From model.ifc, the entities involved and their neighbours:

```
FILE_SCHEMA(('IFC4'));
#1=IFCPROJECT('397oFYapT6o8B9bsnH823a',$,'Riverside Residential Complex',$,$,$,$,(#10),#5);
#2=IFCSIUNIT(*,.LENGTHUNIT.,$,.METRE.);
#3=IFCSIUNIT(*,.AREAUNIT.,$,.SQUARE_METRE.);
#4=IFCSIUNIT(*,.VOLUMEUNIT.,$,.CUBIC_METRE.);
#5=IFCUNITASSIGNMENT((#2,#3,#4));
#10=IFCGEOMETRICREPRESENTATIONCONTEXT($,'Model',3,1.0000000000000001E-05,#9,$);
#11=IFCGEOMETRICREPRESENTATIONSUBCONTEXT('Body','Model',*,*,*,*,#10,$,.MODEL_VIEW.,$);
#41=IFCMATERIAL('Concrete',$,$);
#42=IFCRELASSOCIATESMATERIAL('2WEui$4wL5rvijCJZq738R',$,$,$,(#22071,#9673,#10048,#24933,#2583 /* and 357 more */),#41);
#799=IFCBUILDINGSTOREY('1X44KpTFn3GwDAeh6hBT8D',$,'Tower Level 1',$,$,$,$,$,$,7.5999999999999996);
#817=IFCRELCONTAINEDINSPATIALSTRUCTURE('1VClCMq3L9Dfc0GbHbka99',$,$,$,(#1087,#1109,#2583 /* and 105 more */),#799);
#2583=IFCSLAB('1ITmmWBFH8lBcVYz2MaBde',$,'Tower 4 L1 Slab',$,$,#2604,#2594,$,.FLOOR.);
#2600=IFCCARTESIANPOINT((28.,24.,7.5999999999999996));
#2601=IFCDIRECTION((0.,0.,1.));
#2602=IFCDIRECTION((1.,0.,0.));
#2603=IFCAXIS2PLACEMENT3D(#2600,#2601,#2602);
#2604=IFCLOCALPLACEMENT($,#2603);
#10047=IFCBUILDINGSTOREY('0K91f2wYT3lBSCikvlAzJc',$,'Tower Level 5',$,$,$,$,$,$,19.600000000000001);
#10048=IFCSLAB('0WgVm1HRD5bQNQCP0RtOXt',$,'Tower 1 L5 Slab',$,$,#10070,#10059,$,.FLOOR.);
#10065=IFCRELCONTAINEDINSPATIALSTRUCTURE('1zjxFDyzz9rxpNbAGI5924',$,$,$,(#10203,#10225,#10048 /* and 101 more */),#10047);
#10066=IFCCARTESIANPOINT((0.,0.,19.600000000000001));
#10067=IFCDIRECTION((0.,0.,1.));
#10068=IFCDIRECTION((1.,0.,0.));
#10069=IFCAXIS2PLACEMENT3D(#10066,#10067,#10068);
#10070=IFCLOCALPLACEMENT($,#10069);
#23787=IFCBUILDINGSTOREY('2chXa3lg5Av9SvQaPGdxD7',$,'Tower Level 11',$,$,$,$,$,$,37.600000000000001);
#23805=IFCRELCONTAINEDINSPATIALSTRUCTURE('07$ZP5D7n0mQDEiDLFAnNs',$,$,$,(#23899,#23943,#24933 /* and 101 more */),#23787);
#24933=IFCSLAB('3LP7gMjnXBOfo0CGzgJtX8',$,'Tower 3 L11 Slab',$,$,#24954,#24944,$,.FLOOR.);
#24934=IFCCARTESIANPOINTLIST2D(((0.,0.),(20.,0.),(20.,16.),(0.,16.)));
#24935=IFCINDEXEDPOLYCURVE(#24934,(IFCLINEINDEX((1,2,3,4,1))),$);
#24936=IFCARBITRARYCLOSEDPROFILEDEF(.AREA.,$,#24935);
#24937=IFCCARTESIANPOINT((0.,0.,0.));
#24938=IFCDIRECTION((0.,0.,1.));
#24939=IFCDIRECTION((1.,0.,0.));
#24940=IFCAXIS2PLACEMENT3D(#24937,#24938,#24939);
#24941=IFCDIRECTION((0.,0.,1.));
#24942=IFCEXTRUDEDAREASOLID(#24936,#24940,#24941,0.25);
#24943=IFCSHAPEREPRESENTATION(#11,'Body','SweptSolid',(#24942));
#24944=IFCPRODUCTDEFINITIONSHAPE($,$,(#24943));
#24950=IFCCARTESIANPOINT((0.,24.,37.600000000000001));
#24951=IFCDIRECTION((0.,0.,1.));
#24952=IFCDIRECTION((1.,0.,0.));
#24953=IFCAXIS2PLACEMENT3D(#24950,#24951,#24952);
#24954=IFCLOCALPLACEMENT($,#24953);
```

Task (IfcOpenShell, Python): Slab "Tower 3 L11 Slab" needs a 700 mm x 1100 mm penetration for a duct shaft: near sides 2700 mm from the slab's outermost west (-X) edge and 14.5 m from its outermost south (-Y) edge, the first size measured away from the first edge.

```python
import numpy as np
import ifcopenshell
import ifcopenshell.api.feature
import ifcopenshell.api.geometry
import ifcopenshell.api.root
import ifcopenshell.geom
import ifcopenshell.util.placement
import ifcopenshell.util.representation
import ifcopenshell.util.shape
import ifcopenshell.util.unit

model = ifcopenshell.open("model.ifc")
unit_scale = ifcopenshell.util.unit.calculate_unit_scale(model)
settings = ifcopenshell.geom.settings()


def volume(element):
    """Net volume in cubic metres, openings subtracted."""
    shape = ifcopenshell.geom.create_shape(settings, element)
    return ifcopenshell.util.shape.get_volume(shape.geometry)


slab = model.by_guid("3LP7gMjnXBOfo0CGzgJtX8")
before = volume(slab)

# Extent in the slab's own axes, in metres. The edges named are its -X and -Y sides.
slab_shape = ifcopenshell.geom.create_shape(settings, slab)
vertices = ifcopenshell.util.shape.get_vertices(slab_shape.geometry)
x_min, y_min, bottom = vertices.min(axis=0)
top = vertices[:, 2].max()

opening = ifcopenshell.api.root.create_entity(model, ifc_class="IfcOpeningElement", name="Duct shaft opening", predefined_type="OPENING")
context = ifcopenshell.util.representation.get_context(model, "Model", "Body", "MODEL_VIEW")
width, depth = 0.7, 1.1
outline = [(0.0, 0.0), (width, 0.0), (width, depth), (0.0, depth), (0.0, 0.0)]
# Overshoot both faces by 50 mm so the cut is clean.
shape = ifcopenshell.api.geometry.add_slab_representation(
    model, context=context, depth=top - bottom + 0.1, polyline=outline
)
ifcopenshell.api.geometry.assign_representation(model, product=opening, representation=shape)

matrix = ifcopenshell.util.placement.get_local_placement(slab.ObjectPlacement)
matrix[:, 3] = matrix @ np.append(np.array([x_min + 2.7, y_min + 14.5, bottom - 0.05]) / unit_scale, 1.0)
ifcopenshell.api.geometry.edit_object_placement(model, product=opening, matrix=matrix, is_si=False)
ifcopenshell.api.feature.add_feature(model, feature=opening, element=slab)

after = volume(slab)

print(f"slab volume {before:.3f} -> {after:.3f} m3")

model.write("model_v2.ifc")
```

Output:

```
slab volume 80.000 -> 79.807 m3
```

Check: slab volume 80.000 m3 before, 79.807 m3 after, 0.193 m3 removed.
